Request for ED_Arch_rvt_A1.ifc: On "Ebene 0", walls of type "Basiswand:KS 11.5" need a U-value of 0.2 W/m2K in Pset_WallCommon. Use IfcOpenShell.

First a look at what the model holds.

```python
import ifcopenshell
import ifcopenshell.util.element

model = ifcopenshell.open("ED_Arch_rvt_A1.ifc")
print(model.schema)
storey = next(s for s in model.by_type("IfcBuildingStorey") if s.Name == "Ebene 0")
walls = [e for e in ifcopenshell.util.element.get_decomposition(storey) if e.is_a("IfcWall")]
seen = {}
for e in walls:
    element_type = ifcopenshell.util.element.get_type(e)
    key = (element_type.Name if element_type != e and element_type else None, ifcopenshell.util.element.get_pset(e, "Pset_WallCommon", "ThermalTransmittance"))
    seen[key] = seen.get(key, 0) + 1
for (name, value), count in sorted(seen.items(), key=str):
    print(count, "x", name, "|", value)
```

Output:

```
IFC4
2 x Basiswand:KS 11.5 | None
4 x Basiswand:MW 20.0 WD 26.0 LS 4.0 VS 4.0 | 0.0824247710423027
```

```python
import ifcopenshell
import ifcopenshell.api.pset
import ifcopenshell.util.element

model = ifcopenshell.open("ED_Arch_rvt_A1.ifc")

storey = next(s for s in model.by_type("IfcBuildingStorey") if s.Name == "Ebene 0")
walls = [e for e in ifcopenshell.util.element.get_decomposition(storey) if e.is_a("IfcWall")]

count = 0
for e in walls:
    element_type = ifcopenshell.util.element.get_type(e)
    if element_type in (None, e) or element_type.Name != "Basiswand:KS 11.5":
        continue
    # add_pset returns the element's existing set when there is one.
    pset = ifcopenshell.api.pset.add_pset(model, product=e, name="Pset_WallCommon")
    ifcopenshell.api.pset.edit_pset(model, pset=pset, properties={"ThermalTransmittance": 0.2})
    count += 1

print(count, "walls updated")

model.write("ED_Arch_rvt_A1-out.ifc")
```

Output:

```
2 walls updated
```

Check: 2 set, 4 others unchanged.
